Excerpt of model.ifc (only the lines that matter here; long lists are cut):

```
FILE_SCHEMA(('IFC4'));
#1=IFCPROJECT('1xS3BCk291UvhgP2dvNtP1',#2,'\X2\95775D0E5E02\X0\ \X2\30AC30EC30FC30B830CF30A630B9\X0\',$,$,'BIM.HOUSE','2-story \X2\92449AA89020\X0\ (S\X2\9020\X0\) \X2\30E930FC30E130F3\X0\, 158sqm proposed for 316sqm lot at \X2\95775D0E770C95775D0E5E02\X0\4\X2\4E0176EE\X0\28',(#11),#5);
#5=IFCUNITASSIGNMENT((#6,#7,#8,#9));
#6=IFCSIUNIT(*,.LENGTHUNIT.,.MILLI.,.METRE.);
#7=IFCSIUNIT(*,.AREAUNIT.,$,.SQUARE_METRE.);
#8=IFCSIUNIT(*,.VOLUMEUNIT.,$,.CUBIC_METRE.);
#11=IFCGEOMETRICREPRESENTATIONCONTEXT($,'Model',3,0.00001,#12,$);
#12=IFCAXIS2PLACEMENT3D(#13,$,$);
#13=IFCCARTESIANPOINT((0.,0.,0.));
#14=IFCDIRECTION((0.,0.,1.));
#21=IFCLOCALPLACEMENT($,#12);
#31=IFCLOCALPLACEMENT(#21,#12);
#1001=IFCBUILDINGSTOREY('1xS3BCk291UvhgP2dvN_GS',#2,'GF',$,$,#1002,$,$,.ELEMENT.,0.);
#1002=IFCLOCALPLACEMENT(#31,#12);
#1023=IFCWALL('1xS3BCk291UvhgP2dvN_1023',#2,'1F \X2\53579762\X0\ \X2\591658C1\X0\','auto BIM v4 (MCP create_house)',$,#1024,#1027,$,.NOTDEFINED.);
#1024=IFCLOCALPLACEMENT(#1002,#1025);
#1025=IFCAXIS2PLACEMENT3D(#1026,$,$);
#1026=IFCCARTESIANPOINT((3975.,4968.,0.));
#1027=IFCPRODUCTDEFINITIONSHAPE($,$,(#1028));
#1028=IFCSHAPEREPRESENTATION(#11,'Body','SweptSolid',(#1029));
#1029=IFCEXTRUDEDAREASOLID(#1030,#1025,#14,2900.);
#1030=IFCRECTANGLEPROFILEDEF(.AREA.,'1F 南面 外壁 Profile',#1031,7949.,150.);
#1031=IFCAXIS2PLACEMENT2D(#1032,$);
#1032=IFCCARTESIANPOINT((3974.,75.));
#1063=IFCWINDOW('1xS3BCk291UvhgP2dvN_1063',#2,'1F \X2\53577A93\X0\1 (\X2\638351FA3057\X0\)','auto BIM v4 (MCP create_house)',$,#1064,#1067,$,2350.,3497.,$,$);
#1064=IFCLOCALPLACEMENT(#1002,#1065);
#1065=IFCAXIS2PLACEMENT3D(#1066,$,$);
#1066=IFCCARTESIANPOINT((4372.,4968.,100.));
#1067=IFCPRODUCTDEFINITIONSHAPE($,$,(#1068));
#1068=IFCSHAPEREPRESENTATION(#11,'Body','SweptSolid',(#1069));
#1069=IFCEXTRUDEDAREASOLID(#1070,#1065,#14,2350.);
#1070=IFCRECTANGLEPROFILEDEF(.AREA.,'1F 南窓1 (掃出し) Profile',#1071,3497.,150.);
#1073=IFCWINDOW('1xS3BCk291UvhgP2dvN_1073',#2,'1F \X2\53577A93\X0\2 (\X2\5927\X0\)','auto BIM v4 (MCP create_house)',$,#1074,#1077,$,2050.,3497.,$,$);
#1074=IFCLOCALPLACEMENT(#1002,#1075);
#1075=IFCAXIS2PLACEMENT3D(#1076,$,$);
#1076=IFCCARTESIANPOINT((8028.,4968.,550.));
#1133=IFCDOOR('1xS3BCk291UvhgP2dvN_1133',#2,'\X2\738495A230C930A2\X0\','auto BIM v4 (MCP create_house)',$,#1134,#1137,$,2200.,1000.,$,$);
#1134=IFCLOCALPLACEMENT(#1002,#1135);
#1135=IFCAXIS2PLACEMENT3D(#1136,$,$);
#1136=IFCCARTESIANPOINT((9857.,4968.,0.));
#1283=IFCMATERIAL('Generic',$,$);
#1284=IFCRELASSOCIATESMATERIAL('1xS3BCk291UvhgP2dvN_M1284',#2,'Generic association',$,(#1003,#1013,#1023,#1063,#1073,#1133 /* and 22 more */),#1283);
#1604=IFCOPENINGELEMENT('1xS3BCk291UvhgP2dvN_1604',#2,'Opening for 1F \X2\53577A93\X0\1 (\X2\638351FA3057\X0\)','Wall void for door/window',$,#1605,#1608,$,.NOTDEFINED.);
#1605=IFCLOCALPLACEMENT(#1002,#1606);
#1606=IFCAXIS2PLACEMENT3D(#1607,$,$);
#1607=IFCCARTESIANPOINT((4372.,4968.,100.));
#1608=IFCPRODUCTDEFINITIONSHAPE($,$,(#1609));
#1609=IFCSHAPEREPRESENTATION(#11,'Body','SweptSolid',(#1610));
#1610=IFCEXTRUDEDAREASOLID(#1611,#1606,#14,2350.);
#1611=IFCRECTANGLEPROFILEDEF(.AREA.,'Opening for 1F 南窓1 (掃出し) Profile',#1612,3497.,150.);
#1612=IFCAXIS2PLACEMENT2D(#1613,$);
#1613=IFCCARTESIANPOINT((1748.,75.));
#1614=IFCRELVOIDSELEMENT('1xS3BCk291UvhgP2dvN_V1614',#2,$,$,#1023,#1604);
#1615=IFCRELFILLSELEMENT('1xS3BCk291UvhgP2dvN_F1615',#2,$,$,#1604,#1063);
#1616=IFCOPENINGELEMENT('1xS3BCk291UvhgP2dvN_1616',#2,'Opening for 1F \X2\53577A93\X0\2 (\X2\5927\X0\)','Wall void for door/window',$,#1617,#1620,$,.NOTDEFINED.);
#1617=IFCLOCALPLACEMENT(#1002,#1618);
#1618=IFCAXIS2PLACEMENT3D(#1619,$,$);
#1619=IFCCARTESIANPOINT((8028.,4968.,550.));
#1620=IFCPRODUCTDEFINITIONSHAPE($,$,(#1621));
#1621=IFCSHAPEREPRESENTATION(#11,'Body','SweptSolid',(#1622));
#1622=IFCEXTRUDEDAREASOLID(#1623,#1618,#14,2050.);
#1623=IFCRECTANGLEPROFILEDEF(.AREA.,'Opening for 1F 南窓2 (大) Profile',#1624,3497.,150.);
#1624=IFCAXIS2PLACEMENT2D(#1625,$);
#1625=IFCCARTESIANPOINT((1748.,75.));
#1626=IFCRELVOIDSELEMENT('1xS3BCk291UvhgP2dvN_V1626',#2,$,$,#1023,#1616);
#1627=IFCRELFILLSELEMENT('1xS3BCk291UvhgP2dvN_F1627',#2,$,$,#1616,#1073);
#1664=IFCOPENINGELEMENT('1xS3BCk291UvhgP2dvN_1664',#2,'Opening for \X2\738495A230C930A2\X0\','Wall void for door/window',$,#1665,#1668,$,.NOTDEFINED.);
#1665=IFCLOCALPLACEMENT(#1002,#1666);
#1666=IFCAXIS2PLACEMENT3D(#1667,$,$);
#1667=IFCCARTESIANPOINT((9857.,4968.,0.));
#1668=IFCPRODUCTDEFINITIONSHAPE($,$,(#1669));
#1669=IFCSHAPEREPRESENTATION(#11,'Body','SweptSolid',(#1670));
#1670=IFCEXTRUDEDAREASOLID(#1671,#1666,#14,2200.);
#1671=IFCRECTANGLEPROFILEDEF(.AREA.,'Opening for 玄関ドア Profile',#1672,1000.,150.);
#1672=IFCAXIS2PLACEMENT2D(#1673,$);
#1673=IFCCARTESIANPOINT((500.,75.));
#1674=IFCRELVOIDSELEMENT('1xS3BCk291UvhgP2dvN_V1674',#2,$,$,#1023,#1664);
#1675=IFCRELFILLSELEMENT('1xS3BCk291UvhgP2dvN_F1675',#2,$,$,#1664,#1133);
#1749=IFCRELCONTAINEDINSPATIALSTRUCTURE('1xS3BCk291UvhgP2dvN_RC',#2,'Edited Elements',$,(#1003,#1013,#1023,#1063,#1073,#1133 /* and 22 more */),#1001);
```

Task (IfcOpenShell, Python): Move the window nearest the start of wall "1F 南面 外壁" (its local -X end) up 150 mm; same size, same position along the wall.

```python
import numpy as np
import ifcopenshell
import ifcopenshell.api.geometry
import ifcopenshell.util.placement
import ifcopenshell.util.unit

model = ifcopenshell.open("model.ifc")
unit_scale = ifcopenshell.util.unit.calculate_unit_scale(model)

window = model.by_guid("1xS3BCk291UvhgP2dvN_1063")
opening = window.FillsVoids[0].RelatingOpeningElement
dz = 150.0

shift = np.array([0.0, 0.0, dz])
# The window is not placed relative to its opening, so move both.
for product in (opening, window):
    matrix = ifcopenshell.util.placement.get_local_placement(product.ObjectPlacement)
    matrix[:3, 3] += shift
    ifcopenshell.api.geometry.edit_object_placement(model, product=product, matrix=matrix, is_si=False)

print(f"moved by {dz * unit_scale:+.3f} m")

model.write("model-out.ifc")
```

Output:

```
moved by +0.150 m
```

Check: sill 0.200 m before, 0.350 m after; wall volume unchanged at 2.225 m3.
